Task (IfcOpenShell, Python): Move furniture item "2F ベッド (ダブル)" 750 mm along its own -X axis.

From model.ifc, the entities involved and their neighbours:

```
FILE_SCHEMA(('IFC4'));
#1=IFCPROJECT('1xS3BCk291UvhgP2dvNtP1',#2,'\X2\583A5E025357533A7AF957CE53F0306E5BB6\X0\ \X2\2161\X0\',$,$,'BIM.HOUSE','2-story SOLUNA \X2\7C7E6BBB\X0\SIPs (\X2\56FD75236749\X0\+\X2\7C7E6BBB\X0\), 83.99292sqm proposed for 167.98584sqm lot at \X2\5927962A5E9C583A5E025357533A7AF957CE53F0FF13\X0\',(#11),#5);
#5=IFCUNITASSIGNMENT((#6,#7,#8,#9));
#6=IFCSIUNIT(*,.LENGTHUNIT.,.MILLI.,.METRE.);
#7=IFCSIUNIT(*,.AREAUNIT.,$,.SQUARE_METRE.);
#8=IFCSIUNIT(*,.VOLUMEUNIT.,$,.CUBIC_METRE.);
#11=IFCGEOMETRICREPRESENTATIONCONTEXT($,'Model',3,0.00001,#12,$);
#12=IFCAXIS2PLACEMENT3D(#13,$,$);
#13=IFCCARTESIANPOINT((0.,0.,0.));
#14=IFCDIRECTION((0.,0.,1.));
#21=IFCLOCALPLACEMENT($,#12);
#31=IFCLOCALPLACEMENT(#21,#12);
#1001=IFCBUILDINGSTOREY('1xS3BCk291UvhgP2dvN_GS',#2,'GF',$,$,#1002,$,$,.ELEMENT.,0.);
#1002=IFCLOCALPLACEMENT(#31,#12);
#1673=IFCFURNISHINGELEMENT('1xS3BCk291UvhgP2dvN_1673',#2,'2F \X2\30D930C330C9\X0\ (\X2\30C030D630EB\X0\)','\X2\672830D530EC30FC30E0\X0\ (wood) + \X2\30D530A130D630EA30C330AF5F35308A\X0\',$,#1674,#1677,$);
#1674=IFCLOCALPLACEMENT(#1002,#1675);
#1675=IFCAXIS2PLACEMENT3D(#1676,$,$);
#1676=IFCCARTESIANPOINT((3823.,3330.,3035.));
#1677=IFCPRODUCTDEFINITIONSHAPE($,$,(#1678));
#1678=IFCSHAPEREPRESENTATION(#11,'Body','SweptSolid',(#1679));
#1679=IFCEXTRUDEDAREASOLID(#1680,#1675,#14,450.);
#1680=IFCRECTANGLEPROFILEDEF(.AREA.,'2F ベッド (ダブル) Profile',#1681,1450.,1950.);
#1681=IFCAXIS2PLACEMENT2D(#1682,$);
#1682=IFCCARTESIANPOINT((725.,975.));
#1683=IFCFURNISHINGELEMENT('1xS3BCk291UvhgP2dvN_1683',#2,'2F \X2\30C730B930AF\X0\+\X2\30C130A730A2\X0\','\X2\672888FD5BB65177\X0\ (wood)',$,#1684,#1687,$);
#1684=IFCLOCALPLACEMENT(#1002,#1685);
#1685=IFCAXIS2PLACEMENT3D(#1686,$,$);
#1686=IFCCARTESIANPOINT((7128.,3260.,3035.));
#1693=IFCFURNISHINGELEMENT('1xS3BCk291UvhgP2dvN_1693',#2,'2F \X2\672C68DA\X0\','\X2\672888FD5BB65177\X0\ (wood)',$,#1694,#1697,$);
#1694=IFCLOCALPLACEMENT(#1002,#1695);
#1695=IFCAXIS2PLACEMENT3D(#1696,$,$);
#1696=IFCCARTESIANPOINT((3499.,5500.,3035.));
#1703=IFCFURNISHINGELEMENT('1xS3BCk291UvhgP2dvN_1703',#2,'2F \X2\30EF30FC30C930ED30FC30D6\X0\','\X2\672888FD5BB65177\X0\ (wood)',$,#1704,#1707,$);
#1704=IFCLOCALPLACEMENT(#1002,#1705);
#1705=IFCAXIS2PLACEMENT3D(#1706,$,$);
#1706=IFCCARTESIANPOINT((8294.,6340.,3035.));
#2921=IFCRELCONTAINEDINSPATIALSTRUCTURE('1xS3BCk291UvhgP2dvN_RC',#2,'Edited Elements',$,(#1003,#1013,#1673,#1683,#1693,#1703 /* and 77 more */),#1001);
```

```python
import ifcopenshell
import ifcopenshell.api.geometry
import ifcopenshell.util.placement
import ifcopenshell.util.unit

model = ifcopenshell.open("model.ifc")
unit_scale = ifcopenshell.util.unit.calculate_unit_scale(model)

item = model.by_guid("1xS3BCk291UvhgP2dvN_1673")
matrix = ifcopenshell.util.placement.get_local_placement(item.ObjectPlacement)
matrix[:3, 3] -= matrix[:3, 0] * 0.75 / unit_scale
ifcopenshell.api.geometry.edit_object_placement(model, product=item, matrix=matrix, is_si=False)

print(ifcopenshell.util.placement.get_local_placement(item.ObjectPlacement).round(3) + 0.0)

model.write("model_edited.ifc")
```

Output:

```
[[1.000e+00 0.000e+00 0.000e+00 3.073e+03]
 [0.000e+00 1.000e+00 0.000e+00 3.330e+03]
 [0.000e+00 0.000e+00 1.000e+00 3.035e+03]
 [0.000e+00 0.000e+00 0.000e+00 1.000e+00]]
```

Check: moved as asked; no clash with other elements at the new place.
